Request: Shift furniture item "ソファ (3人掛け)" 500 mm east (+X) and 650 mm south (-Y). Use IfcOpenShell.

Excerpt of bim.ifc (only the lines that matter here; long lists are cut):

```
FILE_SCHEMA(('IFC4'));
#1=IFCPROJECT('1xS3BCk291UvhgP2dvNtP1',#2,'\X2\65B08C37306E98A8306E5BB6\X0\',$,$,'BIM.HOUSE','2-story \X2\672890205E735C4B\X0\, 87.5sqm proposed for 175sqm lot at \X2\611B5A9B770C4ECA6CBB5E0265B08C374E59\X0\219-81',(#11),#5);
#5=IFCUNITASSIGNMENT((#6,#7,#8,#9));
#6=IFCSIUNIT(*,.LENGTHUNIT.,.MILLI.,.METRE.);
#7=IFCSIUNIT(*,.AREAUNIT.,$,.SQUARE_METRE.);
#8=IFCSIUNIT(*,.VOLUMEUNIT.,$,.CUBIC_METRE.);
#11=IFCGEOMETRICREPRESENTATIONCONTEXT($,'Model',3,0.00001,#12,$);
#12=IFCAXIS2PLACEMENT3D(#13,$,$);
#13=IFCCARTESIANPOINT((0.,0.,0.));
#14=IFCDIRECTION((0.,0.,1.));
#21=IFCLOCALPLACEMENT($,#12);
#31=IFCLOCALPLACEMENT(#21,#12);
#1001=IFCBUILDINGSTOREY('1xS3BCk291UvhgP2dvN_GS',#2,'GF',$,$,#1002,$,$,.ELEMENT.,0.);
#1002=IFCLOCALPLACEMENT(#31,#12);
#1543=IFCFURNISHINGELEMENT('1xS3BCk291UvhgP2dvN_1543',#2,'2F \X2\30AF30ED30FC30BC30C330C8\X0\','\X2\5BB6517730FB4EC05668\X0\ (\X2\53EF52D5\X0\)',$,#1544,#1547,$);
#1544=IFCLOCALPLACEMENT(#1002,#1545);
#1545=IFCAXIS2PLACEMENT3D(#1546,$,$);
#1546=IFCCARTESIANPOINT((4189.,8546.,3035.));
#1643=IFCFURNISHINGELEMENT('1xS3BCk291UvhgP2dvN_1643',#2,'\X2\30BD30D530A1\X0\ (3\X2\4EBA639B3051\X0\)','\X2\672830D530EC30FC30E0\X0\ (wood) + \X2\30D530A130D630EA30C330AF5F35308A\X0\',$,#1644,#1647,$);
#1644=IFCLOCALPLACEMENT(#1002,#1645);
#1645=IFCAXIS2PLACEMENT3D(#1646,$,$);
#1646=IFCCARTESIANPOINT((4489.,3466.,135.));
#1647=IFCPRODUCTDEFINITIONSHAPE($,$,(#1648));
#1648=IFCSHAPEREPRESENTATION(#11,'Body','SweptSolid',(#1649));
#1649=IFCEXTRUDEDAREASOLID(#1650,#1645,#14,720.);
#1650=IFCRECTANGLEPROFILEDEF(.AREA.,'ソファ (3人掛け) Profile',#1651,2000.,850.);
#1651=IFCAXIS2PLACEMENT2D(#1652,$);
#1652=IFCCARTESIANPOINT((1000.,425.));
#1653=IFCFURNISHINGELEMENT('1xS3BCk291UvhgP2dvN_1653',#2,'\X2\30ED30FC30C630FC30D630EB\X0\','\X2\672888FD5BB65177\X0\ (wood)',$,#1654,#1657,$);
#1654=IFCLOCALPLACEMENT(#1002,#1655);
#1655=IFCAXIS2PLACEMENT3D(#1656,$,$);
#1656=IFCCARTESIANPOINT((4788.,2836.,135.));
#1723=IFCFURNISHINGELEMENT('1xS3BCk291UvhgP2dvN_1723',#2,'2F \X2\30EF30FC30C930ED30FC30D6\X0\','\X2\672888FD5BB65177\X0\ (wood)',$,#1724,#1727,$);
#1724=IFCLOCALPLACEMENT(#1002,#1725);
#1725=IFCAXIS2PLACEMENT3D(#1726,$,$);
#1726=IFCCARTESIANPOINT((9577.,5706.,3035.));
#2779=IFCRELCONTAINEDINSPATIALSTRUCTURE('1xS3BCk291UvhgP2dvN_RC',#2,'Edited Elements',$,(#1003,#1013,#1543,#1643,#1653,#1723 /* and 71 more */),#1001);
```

```python
import ifcopenshell
import ifcopenshell.api.geometry
import ifcopenshell.util.placement
import ifcopenshell.util.unit

model = ifcopenshell.open("bim.ifc")
unit_scale = ifcopenshell.util.unit.calculate_unit_scale(model)

item = model.by_id(1643)
matrix = ifcopenshell.util.placement.get_local_placement(item.ObjectPlacement)
matrix[0, 3] += 0.5 / unit_scale
matrix[1, 3] -= 0.65 / unit_scale
ifcopenshell.api.geometry.edit_object_placement(model, product=item, matrix=matrix, is_si=False)

print(ifcopenshell.util.placement.get_local_placement(item.ObjectPlacement).round(3) + 0.0)

model.write("bim-out.ifc")
```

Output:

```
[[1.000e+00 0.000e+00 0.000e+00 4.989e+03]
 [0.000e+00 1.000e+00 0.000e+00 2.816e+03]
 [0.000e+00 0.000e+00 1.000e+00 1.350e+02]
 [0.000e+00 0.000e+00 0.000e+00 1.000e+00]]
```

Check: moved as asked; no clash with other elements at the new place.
